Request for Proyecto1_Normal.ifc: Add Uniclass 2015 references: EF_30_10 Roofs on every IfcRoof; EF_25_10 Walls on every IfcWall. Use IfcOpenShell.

First a look at what the model holds.

```python
import ifcopenshell

model = ifcopenshell.open("Proyecto1_Normal.ifc")
print(model.schema)
print("classifications:", [c.Name for c in model.by_type("IfcClassification")])
for ifc_class in ("IfcDoor", "IfcRoof", "IfcStair", "IfcWall", "IfcWindow"):
    print(ifc_class, len(model.by_type(ifc_class)))
```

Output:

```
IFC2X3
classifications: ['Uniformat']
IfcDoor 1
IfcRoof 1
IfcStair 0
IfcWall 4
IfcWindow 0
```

```python
import ifcopenshell
import ifcopenshell.api.classification

model = ifcopenshell.open("Proyecto1_Normal.ifc")

# IFC2X3 requires Source and Edition and has no link from the project to the system.
system = model.create_entity("IfcClassification", Source="NBS", Edition="2015", Name="Uniclass 2015")

codes = {
    "IfcRoof": ("EF_30_10", "Roofs"),
    "IfcWall": ("EF_25_10", "Walls"),
}
for ifc_class, (code, name) in codes.items():
    products = model.by_type(ifc_class)
    ifcopenshell.api.classification.add_reference(
        model, products=products, classification=system, identification=code, name=name
    )
    print(code, len(products))

model.write("Proyecto1_Normal_edited.ifc")
```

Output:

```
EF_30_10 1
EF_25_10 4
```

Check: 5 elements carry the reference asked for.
